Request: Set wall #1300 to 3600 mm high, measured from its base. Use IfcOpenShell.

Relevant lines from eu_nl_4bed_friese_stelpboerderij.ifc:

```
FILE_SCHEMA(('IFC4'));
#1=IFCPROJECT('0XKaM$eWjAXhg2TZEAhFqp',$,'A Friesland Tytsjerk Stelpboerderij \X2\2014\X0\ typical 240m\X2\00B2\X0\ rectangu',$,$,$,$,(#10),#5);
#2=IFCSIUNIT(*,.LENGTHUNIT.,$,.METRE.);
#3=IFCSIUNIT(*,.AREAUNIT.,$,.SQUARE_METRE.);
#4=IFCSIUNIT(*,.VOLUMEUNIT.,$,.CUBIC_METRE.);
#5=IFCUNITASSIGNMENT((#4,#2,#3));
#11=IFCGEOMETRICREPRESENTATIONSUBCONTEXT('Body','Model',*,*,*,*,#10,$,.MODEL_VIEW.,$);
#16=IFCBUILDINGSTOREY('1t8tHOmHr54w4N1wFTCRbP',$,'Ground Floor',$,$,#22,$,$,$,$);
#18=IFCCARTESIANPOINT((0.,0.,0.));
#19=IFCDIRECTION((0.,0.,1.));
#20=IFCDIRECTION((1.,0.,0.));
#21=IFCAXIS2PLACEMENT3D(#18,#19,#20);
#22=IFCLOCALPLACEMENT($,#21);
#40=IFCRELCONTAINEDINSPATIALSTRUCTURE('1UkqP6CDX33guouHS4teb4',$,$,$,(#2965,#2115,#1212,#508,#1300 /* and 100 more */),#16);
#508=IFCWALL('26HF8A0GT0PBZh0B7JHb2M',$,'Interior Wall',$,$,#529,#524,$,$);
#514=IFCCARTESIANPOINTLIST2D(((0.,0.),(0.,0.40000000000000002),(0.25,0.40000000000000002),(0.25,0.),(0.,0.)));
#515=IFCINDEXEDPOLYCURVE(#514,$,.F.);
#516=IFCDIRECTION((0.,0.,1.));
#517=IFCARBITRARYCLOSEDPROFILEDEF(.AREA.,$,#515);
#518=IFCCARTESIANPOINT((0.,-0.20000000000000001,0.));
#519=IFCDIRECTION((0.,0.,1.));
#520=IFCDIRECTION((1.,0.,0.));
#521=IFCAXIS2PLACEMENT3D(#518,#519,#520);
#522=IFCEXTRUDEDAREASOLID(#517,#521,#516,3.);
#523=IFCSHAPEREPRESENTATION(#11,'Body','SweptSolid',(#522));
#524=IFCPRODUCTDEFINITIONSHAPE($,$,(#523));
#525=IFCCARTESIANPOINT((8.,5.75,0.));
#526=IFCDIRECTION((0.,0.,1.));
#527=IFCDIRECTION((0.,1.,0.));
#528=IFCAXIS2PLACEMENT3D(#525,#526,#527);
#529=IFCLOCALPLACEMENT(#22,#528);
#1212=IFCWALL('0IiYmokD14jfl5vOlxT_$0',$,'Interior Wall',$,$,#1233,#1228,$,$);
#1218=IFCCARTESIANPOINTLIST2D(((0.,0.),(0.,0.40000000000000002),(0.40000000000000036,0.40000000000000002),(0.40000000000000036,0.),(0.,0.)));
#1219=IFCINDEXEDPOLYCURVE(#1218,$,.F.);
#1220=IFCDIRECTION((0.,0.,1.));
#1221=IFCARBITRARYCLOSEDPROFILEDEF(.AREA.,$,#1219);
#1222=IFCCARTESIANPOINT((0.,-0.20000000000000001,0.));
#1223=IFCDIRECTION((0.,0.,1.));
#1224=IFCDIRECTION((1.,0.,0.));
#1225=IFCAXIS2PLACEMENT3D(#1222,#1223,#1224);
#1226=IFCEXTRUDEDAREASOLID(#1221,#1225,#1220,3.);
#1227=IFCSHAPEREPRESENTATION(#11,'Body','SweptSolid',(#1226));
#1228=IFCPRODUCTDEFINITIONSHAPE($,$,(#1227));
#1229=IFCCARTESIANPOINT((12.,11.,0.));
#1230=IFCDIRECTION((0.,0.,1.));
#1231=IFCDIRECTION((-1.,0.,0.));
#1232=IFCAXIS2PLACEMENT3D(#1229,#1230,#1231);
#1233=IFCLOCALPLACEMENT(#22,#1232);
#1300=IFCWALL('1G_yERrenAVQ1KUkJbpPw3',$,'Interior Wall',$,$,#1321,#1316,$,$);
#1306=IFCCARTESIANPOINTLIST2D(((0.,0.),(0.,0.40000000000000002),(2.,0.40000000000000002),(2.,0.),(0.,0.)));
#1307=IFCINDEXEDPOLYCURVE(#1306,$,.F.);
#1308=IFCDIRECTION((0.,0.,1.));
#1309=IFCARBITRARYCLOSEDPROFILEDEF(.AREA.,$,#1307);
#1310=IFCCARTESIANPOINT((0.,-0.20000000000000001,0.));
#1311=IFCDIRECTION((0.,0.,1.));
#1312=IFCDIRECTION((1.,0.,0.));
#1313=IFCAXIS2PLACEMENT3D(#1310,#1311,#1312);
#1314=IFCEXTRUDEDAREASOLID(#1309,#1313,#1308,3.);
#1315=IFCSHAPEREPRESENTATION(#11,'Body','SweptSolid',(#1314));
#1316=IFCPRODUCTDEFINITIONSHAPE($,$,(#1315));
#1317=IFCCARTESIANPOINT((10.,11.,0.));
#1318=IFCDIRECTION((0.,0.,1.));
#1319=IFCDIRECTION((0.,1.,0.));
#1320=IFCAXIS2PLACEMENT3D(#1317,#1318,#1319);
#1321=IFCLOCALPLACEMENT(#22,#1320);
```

```python
import ifcopenshell
import ifcopenshell.geom
import ifcopenshell.util.representation
import ifcopenshell.util.shape
import ifcopenshell.util.unit

model = ifcopenshell.open("eu_nl_4bed_friese_stelpboerderij.ifc")
unit_scale = ifcopenshell.util.unit.calculate_unit_scale(model)
settings = ifcopenshell.geom.settings()


def volume(element):
    """Net volume in cubic metres, openings subtracted."""
    shape = ifcopenshell.geom.create_shape(settings, element)
    return ifcopenshell.util.shape.get_volume(shape.geometry)


wall = model.by_guid("1G_yERrenAVQ1KUkJbpPw3")
before = volume(wall)

body = ifcopenshell.util.representation.get_representation(wall, "Model", "Body")
solid = body.Items[0]
old_height = solid.Depth
solid.Depth = 3.6 / unit_scale
after = volume(wall)

print(f"height {old_height:g} -> {solid.Depth:g}, volume {before:.3f} -> {after:.3f} m3")

model.write("eu_nl_4bed_friese_stelpboerderij_updated.ifc")
```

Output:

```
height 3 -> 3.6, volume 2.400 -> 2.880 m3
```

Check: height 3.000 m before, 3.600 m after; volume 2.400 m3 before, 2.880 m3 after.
